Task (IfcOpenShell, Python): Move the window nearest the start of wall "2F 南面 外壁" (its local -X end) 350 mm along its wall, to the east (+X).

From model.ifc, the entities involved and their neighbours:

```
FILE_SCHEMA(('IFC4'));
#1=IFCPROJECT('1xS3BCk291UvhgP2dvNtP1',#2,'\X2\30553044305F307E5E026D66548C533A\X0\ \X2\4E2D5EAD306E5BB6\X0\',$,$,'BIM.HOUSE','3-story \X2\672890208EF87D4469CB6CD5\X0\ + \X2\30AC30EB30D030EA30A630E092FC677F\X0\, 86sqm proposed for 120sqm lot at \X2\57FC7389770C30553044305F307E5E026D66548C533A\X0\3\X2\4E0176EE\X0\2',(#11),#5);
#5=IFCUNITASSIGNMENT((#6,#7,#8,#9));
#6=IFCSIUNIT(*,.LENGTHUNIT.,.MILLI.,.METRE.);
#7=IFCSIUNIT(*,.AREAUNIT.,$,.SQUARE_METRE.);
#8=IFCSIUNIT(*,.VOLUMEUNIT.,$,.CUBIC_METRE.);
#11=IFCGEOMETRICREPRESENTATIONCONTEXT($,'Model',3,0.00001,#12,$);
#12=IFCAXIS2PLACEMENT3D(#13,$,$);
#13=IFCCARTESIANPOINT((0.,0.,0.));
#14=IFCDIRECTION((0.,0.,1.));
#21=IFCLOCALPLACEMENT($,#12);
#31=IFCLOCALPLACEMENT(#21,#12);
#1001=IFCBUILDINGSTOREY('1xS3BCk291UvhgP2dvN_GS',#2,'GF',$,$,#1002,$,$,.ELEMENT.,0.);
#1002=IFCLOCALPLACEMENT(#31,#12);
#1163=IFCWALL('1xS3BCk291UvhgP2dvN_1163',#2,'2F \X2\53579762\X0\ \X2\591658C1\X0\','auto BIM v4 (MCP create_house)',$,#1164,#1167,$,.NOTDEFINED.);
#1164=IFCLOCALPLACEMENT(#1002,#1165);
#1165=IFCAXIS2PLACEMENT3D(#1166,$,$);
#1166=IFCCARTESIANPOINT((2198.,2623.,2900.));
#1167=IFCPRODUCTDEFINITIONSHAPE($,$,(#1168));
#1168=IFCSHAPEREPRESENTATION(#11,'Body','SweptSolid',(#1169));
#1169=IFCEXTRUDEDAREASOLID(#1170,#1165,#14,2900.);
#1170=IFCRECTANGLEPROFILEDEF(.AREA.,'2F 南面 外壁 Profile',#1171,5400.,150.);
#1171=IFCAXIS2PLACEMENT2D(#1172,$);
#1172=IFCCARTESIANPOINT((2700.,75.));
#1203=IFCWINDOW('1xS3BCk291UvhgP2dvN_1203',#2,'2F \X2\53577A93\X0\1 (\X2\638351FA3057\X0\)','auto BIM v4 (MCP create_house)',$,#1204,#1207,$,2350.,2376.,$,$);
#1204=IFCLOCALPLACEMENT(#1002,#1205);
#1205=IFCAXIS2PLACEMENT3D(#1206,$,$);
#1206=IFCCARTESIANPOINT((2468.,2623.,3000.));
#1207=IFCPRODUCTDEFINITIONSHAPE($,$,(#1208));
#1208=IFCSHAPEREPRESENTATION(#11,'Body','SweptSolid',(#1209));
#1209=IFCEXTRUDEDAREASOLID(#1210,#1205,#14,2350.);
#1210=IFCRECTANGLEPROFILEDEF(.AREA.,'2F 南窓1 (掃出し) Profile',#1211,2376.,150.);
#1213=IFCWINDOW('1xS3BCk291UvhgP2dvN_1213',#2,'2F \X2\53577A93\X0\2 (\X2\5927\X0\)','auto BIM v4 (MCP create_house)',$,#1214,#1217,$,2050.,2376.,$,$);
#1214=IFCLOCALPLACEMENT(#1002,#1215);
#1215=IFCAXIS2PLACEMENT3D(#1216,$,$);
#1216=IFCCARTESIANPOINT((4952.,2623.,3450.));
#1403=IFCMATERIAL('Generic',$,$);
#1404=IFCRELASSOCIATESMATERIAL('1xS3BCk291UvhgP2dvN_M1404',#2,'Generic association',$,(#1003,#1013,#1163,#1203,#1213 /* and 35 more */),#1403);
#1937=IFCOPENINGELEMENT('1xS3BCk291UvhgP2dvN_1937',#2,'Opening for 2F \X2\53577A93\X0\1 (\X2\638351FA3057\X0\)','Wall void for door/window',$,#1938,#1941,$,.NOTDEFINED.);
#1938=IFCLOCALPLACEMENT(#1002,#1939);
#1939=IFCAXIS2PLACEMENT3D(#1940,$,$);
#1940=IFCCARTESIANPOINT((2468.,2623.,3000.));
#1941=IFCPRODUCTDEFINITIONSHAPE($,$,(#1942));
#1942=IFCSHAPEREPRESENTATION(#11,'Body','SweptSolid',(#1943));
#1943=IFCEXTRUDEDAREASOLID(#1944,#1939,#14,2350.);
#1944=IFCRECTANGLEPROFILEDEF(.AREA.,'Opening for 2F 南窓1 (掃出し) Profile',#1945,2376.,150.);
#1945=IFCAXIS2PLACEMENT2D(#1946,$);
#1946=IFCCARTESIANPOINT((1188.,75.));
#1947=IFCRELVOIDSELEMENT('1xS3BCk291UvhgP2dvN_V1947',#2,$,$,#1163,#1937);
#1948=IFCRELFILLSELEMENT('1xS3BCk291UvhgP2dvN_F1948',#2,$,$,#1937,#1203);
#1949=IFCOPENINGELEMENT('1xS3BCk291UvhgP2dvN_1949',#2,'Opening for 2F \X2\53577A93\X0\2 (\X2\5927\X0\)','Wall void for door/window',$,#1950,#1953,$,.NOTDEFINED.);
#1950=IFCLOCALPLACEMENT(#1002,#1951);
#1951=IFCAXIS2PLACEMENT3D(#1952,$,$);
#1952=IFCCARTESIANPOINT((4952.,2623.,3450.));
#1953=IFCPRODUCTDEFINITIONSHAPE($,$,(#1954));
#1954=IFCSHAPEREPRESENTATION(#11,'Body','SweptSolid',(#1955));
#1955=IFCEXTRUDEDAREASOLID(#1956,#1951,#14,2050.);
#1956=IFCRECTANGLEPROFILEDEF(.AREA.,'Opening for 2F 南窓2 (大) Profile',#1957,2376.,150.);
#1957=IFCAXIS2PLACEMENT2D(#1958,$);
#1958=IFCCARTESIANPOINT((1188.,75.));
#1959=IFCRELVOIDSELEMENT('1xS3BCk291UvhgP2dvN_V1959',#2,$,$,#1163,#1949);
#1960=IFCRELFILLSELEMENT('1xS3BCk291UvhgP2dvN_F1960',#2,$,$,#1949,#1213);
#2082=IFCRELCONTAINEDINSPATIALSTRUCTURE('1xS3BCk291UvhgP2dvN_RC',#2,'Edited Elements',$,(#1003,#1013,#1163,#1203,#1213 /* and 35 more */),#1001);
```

```python
import ifcopenshell
import ifcopenshell.api.geometry
import ifcopenshell.util.placement

model = ifcopenshell.open("model.ifc")

window = model.by_guid("1xS3BCk291UvhgP2dvN_1203")
opening = window.FillsVoids[0].RelatingOpeningElement
wall = opening.VoidsElements[0].RelatingBuildingElement

wall_matrix = ifcopenshell.util.placement.get_local_placement(wall.ObjectPlacement)
shift = wall_matrix[:3, 0] * 350.0
before = ifcopenshell.util.placement.get_local_placement(window.ObjectPlacement)[:3, 3].copy()

# The window is not placed relative to its opening, so move both.
for product in (opening, window):
    matrix = ifcopenshell.util.placement.get_local_placement(product.ObjectPlacement)
    matrix[:3, 3] += shift
    ifcopenshell.api.geometry.edit_object_placement(model, product=product, matrix=matrix, is_si=False)

after = ifcopenshell.util.placement.get_local_placement(window.ObjectPlacement)[:3, 3]
print("window moved by", (after - before).round(3) + 0.0)

model.write("model_updated.ifc")
```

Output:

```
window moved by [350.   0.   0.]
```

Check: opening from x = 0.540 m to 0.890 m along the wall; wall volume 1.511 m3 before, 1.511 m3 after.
